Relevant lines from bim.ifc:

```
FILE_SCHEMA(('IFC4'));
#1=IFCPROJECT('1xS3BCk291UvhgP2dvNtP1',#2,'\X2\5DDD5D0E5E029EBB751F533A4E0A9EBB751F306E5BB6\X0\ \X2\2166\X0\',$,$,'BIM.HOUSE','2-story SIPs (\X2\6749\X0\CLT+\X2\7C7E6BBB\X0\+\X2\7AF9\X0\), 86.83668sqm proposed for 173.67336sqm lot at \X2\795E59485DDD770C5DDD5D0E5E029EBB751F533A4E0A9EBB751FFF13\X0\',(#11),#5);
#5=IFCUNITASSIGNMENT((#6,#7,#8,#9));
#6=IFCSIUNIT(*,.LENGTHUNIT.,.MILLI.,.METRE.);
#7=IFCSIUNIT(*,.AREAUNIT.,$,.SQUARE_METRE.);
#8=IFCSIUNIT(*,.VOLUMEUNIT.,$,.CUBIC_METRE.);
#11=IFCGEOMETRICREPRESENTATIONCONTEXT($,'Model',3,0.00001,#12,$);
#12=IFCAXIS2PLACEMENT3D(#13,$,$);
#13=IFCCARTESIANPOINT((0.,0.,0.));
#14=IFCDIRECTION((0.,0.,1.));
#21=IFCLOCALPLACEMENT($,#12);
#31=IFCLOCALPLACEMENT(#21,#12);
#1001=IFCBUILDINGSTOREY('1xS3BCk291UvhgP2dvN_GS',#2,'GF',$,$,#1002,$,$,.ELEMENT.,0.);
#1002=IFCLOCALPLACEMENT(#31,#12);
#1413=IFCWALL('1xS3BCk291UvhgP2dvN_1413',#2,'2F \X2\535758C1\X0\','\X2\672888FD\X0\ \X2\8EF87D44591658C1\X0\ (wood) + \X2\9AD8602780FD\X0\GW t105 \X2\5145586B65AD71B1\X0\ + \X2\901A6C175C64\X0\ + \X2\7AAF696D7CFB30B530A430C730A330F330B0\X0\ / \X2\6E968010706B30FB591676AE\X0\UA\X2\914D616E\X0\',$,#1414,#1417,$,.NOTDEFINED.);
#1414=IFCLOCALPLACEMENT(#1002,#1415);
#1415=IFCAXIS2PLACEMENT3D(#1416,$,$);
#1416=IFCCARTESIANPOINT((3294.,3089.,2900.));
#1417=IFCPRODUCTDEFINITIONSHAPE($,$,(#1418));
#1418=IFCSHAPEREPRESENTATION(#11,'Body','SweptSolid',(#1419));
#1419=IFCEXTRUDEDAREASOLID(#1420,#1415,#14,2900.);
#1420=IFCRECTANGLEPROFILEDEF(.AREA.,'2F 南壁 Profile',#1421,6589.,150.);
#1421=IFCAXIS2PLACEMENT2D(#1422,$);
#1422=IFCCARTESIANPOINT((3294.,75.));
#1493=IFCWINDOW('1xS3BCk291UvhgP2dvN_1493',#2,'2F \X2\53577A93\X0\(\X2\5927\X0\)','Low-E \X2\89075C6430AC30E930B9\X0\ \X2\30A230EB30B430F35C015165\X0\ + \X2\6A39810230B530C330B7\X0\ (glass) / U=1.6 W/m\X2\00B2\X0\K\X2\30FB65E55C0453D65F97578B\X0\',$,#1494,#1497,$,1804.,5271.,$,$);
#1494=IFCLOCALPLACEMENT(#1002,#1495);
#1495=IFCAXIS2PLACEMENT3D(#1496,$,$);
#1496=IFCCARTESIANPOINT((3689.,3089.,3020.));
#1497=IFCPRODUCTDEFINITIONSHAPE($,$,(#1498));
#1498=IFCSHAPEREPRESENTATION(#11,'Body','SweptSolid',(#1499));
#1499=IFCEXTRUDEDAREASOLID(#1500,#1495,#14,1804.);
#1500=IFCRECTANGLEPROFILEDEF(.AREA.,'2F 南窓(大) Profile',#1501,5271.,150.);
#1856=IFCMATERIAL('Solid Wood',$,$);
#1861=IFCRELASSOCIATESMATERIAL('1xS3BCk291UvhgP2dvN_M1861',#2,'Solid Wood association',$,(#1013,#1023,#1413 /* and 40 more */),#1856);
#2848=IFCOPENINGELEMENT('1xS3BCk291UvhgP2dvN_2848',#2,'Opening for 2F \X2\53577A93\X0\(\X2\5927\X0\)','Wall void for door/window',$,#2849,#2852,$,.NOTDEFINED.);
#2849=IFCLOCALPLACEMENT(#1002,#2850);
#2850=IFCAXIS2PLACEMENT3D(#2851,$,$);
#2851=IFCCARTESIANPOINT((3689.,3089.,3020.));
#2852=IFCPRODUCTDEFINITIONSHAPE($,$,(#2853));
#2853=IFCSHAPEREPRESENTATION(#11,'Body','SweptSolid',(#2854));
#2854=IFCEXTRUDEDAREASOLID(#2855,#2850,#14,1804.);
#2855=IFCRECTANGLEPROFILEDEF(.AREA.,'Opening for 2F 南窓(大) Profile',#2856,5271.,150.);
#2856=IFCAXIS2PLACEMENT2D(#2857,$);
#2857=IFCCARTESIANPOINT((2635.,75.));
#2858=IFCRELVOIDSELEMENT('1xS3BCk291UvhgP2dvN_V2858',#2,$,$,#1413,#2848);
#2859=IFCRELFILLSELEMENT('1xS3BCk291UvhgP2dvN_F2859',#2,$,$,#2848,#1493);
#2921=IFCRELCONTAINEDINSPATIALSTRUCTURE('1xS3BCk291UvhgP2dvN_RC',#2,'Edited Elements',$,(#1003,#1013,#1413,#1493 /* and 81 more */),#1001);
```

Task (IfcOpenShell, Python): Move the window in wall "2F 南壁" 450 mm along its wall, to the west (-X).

```python
import ifcopenshell
import ifcopenshell.api.geometry
import ifcopenshell.util.placement

model = ifcopenshell.open("bim.ifc")

window = model.by_guid("1xS3BCk291UvhgP2dvN_1493")
opening = window.FillsVoids[0].RelatingOpeningElement
wall = opening.VoidsElements[0].RelatingBuildingElement

wall_matrix = ifcopenshell.util.placement.get_local_placement(wall.ObjectPlacement)
shift = wall_matrix[:3, 0] * -450.0
before = ifcopenshell.util.placement.get_local_placement(window.ObjectPlacement)[:3, 3].copy()

# The window is not placed relative to its opening, so move both.
for product in (opening, window):
    matrix = ifcopenshell.util.placement.get_local_placement(product.ObjectPlacement)
    matrix[:3, 3] += shift
    ifcopenshell.api.geometry.edit_object_placement(model, product=product, matrix=matrix, is_si=False)

after = ifcopenshell.util.placement.get_local_placement(window.ObjectPlacement)[:3, 3]
print("window moved by", (after - before).round(3) + 0.0)

model.write("bim-out.ifc")
```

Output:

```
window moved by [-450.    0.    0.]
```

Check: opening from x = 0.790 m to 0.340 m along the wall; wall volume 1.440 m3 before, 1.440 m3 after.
